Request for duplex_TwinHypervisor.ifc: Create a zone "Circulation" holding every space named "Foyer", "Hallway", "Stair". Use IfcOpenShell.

First a look at what the model holds.

```python
import ifcopenshell

model = ifcopenshell.open("duplex_TwinHypervisor.ifc")
print(model.schema)
seen = {}
for space in model.by_type("IfcSpace"):
    seen[space.LongName] = seen.get(space.LongName, 0) + 1
for name, count in sorted(seen.items(), key=str):
    print(count, "x", name)
print("zones:", [z.Name for z in model.by_type("IfcZone")][:20])
```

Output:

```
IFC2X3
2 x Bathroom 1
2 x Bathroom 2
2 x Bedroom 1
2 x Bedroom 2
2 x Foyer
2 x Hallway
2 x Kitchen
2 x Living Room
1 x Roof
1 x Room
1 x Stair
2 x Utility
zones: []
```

```python
import ifcopenshell
import ifcopenshell.api.group
import ifcopenshell.api.root

model = ifcopenshell.open("duplex_TwinHypervisor.ifc")

names = {"Foyer", "Hallway", "Stair"}
spaces = [s for s in model.by_type("IfcSpace") if s.LongName in names]

zone = ifcopenshell.api.root.create_entity(model, ifc_class="IfcZone", name="Circulation")
ifcopenshell.api.group.assign_group(model, products=spaces, group=zone)
print(len(spaces), "spaces in", zone.Name)

model.write("duplex_TwinHypervisor_v2.ifc")
```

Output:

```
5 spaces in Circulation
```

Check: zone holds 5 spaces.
